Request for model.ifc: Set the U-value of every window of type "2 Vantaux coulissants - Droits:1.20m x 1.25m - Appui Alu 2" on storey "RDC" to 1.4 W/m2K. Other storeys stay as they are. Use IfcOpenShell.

First a look at what the model holds.

```python
import ifcopenshell
import ifcopenshell.util.element

model = ifcopenshell.open("model.ifc")
print(model.schema)
storey = next(s for s in model.by_type("IfcBuildingStorey") if s.Name == "RDC")
windows = [e for e in ifcopenshell.util.element.get_decomposition(storey) if e.is_a("IfcWindow")]
seen = {}
for e in windows:
    element_type = ifcopenshell.util.element.get_type(e)
    key = (element_type.Name if element_type != e and element_type else None, ifcopenshell.util.element.get_pset(e, "Pset_WindowCommon", "ThermalTransmittance"))
    seen[key] = seen.get(key, 0) + 1
for (name, value), count in sorted(seen.items(), key=str):
    print(count, "x", name, "|", value)
```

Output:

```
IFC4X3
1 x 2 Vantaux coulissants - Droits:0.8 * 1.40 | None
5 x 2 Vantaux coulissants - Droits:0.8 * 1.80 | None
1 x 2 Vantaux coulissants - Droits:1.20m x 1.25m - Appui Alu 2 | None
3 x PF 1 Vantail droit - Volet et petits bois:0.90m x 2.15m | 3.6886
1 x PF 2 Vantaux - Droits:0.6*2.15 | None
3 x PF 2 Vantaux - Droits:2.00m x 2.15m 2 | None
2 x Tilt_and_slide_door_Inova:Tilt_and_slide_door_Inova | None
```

```python
import ifcopenshell
import ifcopenshell.api.pset
import ifcopenshell.util.element

model = ifcopenshell.open("model.ifc")

storey = next(s for s in model.by_type("IfcBuildingStorey") if s.Name == "RDC")
windows = [e for e in ifcopenshell.util.element.get_decomposition(storey) if e.is_a("IfcWindow")]

count = 0
for e in windows:
    element_type = ifcopenshell.util.element.get_type(e)
    if element_type in (None, e) or element_type.Name != "2 Vantaux coulissants - Droits:1.20m x 1.25m - Appui Alu 2":
        continue
    # add_pset returns the element's existing set when there is one.
    pset = ifcopenshell.api.pset.add_pset(model, product=e, name="Pset_WindowCommon")
    ifcopenshell.api.pset.edit_pset(model, pset=pset, properties={"ThermalTransmittance": 1.4})
    count += 1

print(count, "windows updated")

model.write("model_rev.ifc")
```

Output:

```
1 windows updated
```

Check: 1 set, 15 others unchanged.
